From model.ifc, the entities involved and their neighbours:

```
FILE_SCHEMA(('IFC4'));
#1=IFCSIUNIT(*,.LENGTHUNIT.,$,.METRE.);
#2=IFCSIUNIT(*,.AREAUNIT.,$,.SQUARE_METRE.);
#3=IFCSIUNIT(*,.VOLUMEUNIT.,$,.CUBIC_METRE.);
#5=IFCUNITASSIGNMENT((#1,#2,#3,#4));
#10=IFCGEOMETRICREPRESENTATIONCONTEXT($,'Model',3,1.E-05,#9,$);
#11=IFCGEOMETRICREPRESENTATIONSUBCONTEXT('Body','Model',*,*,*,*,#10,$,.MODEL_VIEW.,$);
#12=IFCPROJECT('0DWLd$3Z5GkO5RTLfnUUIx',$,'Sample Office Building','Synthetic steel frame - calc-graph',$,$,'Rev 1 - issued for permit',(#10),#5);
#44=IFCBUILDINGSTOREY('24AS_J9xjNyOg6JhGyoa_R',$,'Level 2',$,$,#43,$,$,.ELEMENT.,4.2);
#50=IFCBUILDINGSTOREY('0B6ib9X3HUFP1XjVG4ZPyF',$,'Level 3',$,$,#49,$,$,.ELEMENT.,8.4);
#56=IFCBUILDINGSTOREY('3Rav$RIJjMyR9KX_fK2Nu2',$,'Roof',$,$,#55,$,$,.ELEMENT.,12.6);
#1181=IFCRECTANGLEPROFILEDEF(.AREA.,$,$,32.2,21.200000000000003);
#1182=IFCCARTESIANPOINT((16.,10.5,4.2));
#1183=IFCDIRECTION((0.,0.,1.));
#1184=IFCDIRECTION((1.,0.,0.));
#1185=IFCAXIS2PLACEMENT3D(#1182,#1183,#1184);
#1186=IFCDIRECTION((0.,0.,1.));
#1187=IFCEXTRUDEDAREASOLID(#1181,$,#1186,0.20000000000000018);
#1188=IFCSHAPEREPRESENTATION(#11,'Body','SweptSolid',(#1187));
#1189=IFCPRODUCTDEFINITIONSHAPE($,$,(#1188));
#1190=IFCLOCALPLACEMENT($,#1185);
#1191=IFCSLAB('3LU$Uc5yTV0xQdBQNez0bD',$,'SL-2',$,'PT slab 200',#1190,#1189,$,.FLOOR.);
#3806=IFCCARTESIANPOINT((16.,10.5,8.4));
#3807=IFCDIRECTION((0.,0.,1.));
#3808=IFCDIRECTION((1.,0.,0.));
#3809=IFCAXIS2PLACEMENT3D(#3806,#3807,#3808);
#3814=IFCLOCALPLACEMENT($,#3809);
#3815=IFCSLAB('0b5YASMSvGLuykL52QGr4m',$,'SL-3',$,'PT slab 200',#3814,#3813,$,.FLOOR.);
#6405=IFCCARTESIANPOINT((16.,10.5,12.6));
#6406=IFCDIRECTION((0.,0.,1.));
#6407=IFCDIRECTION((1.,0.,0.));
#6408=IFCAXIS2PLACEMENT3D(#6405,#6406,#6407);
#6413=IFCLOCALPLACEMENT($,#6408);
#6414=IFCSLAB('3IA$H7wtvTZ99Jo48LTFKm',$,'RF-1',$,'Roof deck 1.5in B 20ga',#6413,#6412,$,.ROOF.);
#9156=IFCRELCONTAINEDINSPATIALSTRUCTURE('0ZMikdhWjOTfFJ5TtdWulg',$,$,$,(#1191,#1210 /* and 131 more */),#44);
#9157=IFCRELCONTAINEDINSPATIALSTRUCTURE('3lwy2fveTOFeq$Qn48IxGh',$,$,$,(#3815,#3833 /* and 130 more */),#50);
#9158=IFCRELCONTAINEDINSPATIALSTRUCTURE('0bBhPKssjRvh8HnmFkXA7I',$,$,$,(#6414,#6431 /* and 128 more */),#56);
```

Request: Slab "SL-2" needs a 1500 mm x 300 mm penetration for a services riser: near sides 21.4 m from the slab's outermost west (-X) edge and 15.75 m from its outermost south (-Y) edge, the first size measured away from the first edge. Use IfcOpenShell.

```python
import numpy as np
import ifcopenshell
import ifcopenshell.api.feature
import ifcopenshell.api.geometry
import ifcopenshell.api.root
import ifcopenshell.geom
import ifcopenshell.util.placement
import ifcopenshell.util.representation
import ifcopenshell.util.shape
import ifcopenshell.util.unit

model = ifcopenshell.open("model.ifc")
unit_scale = ifcopenshell.util.unit.calculate_unit_scale(model)
settings = ifcopenshell.geom.settings()


def volume(element):
    """Net volume in cubic metres, openings subtracted."""
    shape = ifcopenshell.geom.create_shape(settings, element)
    return ifcopenshell.util.shape.get_volume(shape.geometry)


slab = model.by_id(1191)
before = volume(slab)

# Extent in the slab's own axes, in metres. The edges named are its -X and -Y sides.
slab_shape = ifcopenshell.geom.create_shape(settings, slab)
vertices = ifcopenshell.util.shape.get_vertices(slab_shape.geometry)
x_min, y_min, bottom = vertices.min(axis=0)
top = vertices[:, 2].max()

opening = ifcopenshell.api.root.create_entity(model, ifc_class="IfcOpeningElement", name="Services riser opening", predefined_type="OPENING")
context = ifcopenshell.util.representation.get_context(model, "Model", "Body", "MODEL_VIEW")
width, depth = 1.5, 0.3
outline = [(0.0, 0.0), (width, 0.0), (width, depth), (0.0, depth), (0.0, 0.0)]
# Overshoot both faces by 50 mm so the cut is clean.
shape = ifcopenshell.api.geometry.add_slab_representation(
    model, context=context, depth=top - bottom + 0.1, polyline=outline
)
ifcopenshell.api.geometry.assign_representation(model, product=opening, representation=shape)

matrix = ifcopenshell.util.placement.get_local_placement(slab.ObjectPlacement)
matrix[:, 3] = matrix @ np.append(np.array([x_min + 21.4, y_min + 15.75, bottom - 0.05]) / unit_scale, 1.0)
ifcopenshell.api.geometry.edit_object_placement(model, product=opening, matrix=matrix, is_si=False)
ifcopenshell.api.feature.add_feature(model, feature=opening, element=slab)

after = volume(slab)

print(f"slab volume {before:.3f} -> {after:.3f} m3")

model.write("model_edited.ifc")
```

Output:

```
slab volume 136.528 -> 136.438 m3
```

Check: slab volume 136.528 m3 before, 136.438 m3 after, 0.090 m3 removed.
